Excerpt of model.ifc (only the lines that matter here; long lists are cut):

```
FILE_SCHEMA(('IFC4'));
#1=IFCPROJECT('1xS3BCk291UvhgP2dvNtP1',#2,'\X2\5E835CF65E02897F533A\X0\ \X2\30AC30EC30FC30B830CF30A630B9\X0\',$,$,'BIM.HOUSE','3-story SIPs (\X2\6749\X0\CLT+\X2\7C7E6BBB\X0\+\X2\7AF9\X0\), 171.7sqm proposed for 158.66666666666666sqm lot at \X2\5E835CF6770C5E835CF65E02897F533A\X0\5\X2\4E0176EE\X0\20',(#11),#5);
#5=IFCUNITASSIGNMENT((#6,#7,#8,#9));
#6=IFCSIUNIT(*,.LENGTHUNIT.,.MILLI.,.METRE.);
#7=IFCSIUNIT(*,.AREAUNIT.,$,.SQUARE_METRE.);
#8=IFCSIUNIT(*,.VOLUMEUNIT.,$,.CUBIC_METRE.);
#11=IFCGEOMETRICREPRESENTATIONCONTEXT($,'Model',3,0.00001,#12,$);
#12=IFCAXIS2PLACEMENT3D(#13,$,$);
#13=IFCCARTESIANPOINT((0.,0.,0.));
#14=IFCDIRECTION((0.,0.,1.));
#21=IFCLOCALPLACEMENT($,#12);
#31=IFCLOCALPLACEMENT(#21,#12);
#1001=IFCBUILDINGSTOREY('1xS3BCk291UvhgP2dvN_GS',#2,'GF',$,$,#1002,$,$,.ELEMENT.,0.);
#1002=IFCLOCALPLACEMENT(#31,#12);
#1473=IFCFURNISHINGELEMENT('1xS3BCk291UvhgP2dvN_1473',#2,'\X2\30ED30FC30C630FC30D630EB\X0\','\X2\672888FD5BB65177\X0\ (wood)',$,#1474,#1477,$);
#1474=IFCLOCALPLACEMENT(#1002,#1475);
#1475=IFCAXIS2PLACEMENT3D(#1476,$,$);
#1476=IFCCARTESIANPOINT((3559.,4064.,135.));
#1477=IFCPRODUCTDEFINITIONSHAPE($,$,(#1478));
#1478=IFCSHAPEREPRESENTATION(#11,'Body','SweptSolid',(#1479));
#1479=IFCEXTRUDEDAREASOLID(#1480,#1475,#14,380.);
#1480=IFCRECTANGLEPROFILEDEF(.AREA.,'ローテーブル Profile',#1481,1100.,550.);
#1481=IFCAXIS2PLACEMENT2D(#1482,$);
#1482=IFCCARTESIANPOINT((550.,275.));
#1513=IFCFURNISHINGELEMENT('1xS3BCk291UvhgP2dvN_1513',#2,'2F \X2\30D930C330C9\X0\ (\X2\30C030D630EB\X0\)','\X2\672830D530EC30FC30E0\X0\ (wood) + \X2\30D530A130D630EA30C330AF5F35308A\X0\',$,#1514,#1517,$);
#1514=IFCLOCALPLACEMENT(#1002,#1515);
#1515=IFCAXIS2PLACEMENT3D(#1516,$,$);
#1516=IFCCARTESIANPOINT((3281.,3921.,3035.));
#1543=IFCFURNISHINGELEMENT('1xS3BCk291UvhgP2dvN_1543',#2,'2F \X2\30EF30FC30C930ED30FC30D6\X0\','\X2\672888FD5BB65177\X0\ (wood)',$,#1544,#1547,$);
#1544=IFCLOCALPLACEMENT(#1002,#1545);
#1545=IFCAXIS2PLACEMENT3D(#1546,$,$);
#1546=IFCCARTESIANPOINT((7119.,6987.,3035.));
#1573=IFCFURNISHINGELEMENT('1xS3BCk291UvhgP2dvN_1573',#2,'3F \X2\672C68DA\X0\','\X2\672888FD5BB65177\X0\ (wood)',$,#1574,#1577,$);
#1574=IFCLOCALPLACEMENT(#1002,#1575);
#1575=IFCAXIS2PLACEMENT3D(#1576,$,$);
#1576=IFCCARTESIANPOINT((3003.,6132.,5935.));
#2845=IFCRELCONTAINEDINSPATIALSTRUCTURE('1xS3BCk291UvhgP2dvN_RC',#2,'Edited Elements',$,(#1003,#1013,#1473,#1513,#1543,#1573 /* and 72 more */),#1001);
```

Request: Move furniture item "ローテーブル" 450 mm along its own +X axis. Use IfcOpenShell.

```python
import ifcopenshell
import ifcopenshell.api.geometry
import ifcopenshell.util.placement

model = ifcopenshell.open("model.ifc")

item = model.by_guid("1xS3BCk291UvhgP2dvN_1473")
matrix = ifcopenshell.util.placement.get_local_placement(item.ObjectPlacement)
matrix[:3, 3] += matrix[:3, 0] * 450.0
ifcopenshell.api.geometry.edit_object_placement(model, product=item, matrix=matrix, is_si=False)

print(ifcopenshell.util.placement.get_local_placement(item.ObjectPlacement).round(3) + 0.0)

model.write("model_edited.ifc")
```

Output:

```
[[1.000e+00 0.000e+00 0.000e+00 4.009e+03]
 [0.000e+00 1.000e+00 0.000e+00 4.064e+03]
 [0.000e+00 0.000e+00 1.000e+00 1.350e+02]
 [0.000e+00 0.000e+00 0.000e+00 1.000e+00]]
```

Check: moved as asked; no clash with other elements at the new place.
